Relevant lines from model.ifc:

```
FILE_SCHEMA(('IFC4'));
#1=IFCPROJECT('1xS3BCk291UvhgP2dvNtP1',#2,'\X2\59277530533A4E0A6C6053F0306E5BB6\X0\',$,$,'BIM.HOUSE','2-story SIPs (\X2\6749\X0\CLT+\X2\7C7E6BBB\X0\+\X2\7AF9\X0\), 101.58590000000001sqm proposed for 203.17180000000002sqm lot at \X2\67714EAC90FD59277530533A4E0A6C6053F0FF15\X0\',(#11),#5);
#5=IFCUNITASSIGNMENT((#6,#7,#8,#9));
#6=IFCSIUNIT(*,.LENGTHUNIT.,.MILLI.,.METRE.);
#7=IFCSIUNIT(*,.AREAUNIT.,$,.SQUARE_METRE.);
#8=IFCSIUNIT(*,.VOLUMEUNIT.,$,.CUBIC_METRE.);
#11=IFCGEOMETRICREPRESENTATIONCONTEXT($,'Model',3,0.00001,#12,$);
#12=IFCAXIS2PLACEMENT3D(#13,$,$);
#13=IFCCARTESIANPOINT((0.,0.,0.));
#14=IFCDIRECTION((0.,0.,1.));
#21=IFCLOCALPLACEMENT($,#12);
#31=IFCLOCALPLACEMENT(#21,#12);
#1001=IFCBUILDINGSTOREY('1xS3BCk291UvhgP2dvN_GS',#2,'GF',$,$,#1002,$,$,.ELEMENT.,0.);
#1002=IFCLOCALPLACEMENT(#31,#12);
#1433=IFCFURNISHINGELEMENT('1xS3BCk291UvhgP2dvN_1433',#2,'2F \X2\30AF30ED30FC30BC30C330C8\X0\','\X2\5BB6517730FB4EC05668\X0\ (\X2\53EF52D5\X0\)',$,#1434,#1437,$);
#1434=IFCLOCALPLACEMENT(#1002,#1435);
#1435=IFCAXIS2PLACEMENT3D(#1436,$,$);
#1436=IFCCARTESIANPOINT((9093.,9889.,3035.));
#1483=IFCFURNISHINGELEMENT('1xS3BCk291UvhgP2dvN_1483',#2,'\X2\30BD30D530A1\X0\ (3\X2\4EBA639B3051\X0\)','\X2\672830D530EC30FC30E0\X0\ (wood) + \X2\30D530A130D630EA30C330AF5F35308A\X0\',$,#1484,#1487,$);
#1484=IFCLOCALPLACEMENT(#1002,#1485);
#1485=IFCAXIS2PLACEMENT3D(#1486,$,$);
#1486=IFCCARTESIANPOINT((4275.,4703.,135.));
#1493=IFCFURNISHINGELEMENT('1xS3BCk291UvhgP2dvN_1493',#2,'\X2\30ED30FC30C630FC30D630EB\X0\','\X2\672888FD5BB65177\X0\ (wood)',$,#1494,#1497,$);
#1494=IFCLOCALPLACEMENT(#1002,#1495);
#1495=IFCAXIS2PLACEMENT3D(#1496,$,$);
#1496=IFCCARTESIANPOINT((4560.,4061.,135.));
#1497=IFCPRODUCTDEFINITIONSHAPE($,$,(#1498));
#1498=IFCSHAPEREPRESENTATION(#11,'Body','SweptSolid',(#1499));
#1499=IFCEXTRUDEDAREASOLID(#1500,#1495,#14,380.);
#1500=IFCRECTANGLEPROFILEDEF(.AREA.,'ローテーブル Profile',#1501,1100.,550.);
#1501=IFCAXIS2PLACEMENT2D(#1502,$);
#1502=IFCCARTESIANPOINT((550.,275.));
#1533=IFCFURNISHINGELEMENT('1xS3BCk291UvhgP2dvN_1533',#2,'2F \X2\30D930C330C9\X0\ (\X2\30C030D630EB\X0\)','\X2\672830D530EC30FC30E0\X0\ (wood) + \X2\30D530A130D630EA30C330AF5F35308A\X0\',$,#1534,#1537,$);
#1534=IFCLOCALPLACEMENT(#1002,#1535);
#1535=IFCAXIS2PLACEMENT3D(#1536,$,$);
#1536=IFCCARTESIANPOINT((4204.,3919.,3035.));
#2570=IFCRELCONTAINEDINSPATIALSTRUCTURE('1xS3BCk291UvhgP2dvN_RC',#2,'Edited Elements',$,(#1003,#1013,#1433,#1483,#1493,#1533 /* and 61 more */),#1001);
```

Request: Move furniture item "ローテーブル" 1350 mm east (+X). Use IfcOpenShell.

```python
import ifcopenshell
import ifcopenshell.api.geometry
import ifcopenshell.util.placement
import ifcopenshell.util.unit

model = ifcopenshell.open("model.ifc")
unit_scale = ifcopenshell.util.unit.calculate_unit_scale(model)

item = model.by_guid("1xS3BCk291UvhgP2dvN_1493")
matrix = ifcopenshell.util.placement.get_local_placement(item.ObjectPlacement)
matrix[0, 3] += 1.35 / unit_scale
ifcopenshell.api.geometry.edit_object_placement(model, product=item, matrix=matrix, is_si=False)

print(ifcopenshell.util.placement.get_local_placement(item.ObjectPlacement).round(3) + 0.0)

model.write("model-out.ifc")
```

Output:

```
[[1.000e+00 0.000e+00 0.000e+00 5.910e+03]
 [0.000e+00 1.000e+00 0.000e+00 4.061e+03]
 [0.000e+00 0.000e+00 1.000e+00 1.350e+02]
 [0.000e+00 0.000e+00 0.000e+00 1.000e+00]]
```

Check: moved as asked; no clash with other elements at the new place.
